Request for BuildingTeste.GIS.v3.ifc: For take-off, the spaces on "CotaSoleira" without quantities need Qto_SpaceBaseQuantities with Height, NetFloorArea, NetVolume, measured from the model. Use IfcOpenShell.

First a look at what the model holds.

```python
import ifcopenshell
import ifcopenshell.util.element
import ifcopenshell.util.unit

model = ifcopenshell.open("BuildingTeste.GIS.v3.ifc")
print(model.schema)
for unit_type in ("LENGTHUNIT", "AREAUNIT", "VOLUMEUNIT"):
    print(unit_type, ifcopenshell.util.unit.calculate_unit_scale(model, unit_type))
storey = next(s for s in model.by_type("IfcBuildingStorey") if s.Name == "CotaSoleira")
spaces = [e for e in ifcopenshell.util.element.get_decomposition(storey) if e.is_a("IfcSpace")]
for e in sorted(spaces, key=lambda e: e.id()):
    print(e.id(), e.is_a(), e.Name, list(ifcopenshell.util.element.get_psets(e, qtos_only=True)), sep=" | ")
```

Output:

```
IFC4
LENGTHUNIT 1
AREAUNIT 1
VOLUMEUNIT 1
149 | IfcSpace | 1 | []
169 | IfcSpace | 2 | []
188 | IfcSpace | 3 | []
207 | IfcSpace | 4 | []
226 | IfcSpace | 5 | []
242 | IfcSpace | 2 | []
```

```python
import ifcopenshell
import ifcopenshell.api.pset
import ifcopenshell.geom
import ifcopenshell.util.element
import ifcopenshell.util.shape
import ifcopenshell.util.unit

model = ifcopenshell.open("BuildingTeste.GIS.v3.ifc")
unit_scale = ifcopenshell.util.unit.calculate_unit_scale(model)
area_scale = ifcopenshell.util.unit.calculate_unit_scale(model, "AREAUNIT")
volume_scale = ifcopenshell.util.unit.calculate_unit_scale(model, "VOLUMEUNIT")
settings = ifcopenshell.geom.settings()

storey = next(s for s in model.by_type("IfcBuildingStorey") if s.Name == "CotaSoleira")
spaces = [e for e in ifcopenshell.util.element.get_decomposition(storey) if e.is_a("IfcSpace")]

for e in sorted(spaces, key=lambda e: e.id()):
    if ifcopenshell.util.element.get_psets(e, qtos_only=True, should_inherit=False):
        continue
    # Geometry comes back in metres, in the element's own axes.
    shape = ifcopenshell.geom.create_shape(settings, e)
    values = {
        "Height": ifcopenshell.util.shape.get_z(shape.geometry) / unit_scale,
        "NetFloorArea": ifcopenshell.util.shape.get_footprint_area(shape.geometry) / area_scale,
        "NetVolume": ifcopenshell.util.shape.get_volume(shape.geometry) / volume_scale,
    }
    qto = ifcopenshell.api.pset.add_qto(model, product=e, name="Qto_SpaceBaseQuantities")
    ifcopenshell.api.pset.edit_qto(model, qto=qto, properties=values)
    print(e.id(), {k: round(v, 3) for k, v in values.items()})

model.write("BuildingTeste.GIS.v3_v2.ifc")
```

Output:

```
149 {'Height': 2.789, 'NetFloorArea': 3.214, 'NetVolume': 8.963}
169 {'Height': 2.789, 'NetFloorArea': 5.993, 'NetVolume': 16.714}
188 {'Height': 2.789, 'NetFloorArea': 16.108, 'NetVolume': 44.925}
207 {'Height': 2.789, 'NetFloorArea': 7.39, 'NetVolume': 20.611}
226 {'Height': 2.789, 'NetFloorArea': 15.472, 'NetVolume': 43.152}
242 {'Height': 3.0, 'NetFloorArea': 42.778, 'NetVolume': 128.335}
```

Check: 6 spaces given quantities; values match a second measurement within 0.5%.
